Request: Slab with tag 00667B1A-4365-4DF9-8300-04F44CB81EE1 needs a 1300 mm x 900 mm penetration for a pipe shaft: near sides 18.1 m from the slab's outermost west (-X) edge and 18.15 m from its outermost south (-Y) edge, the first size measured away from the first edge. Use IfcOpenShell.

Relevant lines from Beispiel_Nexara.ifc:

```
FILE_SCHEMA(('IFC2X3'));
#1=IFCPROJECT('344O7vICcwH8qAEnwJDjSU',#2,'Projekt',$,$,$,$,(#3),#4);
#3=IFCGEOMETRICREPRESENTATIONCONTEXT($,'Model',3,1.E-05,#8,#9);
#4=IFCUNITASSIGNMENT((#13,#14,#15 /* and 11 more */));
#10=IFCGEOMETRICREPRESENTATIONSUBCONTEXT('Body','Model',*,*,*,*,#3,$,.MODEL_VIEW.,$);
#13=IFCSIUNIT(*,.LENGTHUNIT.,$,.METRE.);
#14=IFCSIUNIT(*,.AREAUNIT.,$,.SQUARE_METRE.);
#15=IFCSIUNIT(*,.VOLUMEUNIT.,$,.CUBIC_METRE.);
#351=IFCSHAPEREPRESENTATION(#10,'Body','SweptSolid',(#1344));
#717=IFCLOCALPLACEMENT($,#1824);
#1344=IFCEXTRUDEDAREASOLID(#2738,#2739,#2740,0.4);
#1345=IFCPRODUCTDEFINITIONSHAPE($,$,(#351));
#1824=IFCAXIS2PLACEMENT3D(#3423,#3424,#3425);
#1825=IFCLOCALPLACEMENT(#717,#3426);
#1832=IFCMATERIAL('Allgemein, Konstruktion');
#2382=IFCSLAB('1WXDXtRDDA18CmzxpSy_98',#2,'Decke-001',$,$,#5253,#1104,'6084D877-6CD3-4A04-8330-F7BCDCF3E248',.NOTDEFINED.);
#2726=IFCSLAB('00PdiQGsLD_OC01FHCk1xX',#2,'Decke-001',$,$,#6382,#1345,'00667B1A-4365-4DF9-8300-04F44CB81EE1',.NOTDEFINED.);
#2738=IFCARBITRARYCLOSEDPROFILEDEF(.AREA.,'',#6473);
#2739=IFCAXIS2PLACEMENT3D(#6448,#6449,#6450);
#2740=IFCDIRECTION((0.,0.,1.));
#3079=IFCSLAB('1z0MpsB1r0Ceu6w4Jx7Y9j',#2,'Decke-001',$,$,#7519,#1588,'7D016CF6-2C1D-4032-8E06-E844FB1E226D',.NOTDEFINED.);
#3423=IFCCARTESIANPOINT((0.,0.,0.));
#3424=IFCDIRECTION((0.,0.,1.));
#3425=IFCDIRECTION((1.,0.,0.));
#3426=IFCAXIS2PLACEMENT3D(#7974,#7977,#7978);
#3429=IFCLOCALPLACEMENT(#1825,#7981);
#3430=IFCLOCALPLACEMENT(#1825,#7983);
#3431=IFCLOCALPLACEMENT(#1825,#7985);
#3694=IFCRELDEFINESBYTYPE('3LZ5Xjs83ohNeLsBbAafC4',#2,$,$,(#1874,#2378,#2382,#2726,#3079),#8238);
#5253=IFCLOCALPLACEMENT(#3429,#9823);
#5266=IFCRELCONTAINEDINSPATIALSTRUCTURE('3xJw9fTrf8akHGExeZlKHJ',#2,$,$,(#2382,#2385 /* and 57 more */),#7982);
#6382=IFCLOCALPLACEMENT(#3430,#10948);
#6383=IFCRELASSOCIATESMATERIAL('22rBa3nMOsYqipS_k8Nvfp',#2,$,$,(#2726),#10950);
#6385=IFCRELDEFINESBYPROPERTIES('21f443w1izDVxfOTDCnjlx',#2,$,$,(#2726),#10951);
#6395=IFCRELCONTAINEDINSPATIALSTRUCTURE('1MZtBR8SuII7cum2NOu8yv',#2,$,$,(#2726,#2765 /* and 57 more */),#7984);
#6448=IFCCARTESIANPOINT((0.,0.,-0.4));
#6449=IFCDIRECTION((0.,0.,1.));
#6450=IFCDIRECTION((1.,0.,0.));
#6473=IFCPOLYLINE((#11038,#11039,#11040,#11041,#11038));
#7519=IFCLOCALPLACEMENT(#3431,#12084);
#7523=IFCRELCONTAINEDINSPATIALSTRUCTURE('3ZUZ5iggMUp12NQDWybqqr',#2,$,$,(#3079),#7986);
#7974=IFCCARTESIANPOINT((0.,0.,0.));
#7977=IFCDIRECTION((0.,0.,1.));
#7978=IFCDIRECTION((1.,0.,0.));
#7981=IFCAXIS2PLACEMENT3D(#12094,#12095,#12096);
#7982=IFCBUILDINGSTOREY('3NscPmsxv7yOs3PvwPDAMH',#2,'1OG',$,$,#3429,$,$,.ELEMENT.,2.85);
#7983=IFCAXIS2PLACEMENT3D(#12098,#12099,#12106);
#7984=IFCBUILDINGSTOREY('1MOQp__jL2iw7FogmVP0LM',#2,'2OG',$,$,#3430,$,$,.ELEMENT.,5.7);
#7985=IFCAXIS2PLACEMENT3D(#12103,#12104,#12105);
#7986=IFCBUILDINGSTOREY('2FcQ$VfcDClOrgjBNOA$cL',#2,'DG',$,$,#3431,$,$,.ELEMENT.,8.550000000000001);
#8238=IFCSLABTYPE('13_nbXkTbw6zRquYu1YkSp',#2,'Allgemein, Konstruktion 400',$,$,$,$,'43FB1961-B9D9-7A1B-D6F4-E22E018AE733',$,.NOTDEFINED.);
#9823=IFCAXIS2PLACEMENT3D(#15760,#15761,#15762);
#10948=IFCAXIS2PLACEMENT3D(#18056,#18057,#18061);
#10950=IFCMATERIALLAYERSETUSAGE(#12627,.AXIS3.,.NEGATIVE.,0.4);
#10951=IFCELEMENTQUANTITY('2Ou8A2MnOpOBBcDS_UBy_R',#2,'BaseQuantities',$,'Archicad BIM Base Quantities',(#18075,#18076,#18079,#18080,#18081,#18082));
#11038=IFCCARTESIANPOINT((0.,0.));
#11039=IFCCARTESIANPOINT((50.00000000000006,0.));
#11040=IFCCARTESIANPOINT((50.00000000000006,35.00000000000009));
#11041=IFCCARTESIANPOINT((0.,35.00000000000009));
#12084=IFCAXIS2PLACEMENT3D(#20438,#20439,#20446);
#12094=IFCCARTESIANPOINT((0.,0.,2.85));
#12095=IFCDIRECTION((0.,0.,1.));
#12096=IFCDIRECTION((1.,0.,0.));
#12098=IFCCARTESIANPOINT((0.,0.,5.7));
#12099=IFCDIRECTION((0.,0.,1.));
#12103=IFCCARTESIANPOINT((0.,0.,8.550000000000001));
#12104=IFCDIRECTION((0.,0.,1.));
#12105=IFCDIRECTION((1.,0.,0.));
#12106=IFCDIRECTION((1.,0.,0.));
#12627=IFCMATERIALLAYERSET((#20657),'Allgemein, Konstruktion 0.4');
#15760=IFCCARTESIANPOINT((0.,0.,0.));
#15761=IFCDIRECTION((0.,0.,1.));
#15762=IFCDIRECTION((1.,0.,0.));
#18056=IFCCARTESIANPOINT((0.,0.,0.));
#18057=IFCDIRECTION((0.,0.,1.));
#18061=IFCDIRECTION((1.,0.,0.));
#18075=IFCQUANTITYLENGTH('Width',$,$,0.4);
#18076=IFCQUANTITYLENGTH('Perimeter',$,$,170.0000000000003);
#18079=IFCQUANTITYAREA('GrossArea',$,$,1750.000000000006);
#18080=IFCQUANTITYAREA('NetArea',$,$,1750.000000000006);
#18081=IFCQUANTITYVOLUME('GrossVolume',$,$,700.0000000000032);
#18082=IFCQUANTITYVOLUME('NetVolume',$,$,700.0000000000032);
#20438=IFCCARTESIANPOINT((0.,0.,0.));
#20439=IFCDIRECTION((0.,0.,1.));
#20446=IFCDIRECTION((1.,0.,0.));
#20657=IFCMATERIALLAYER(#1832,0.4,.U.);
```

```python
import numpy as np
import ifcopenshell
import ifcopenshell.api.feature
import ifcopenshell.api.geometry
import ifcopenshell.api.pset
import ifcopenshell.api.root
import ifcopenshell.geom
import ifcopenshell.util.element
import ifcopenshell.util.placement
import ifcopenshell.util.representation
import ifcopenshell.util.shape
import ifcopenshell.util.unit

model = ifcopenshell.open("Beispiel_Nexara.ifc")
unit_scale = ifcopenshell.util.unit.calculate_unit_scale(model)
area_scale = ifcopenshell.util.unit.calculate_unit_scale(model, "AREAUNIT")
volume_scale = ifcopenshell.util.unit.calculate_unit_scale(model, "VOLUMEUNIT")
settings = ifcopenshell.geom.settings()


def volume(element):
    """Net volume in cubic metres, openings subtracted."""
    shape = ifcopenshell.geom.create_shape(settings, element)
    return ifcopenshell.util.shape.get_volume(shape.geometry)


slab = model.by_guid("00PdiQGsLD_OC01FHCk1xX")
before = volume(slab)

# Extent in the slab's own axes, in metres. The edges named are its -X and -Y sides.
slab_shape = ifcopenshell.geom.create_shape(settings, slab)
vertices = ifcopenshell.util.shape.get_vertices(slab_shape.geometry)
x_min, y_min, bottom = vertices.min(axis=0)
top = vertices[:, 2].max()

opening = ifcopenshell.api.root.create_entity(model, ifc_class="IfcOpeningElement", name="Pipe shaft opening")
context = ifcopenshell.util.representation.get_context(model, "Model", "Body", "MODEL_VIEW")
width, depth = 1.3, 0.9
outline = [(0.0, 0.0), (width, 0.0), (width, depth), (0.0, depth), (0.0, 0.0)]
# Overshoot both faces by 50 mm so the cut is clean.
shape = ifcopenshell.api.geometry.add_slab_representation(
    model, context=context, depth=top - bottom + 0.1, polyline=outline
)
ifcopenshell.api.geometry.assign_representation(model, product=opening, representation=shape)

matrix = ifcopenshell.util.placement.get_local_placement(slab.ObjectPlacement)
matrix[:, 3] = matrix @ np.append(np.array([x_min + 18.1, y_min + 18.15, bottom - 0.05]) / unit_scale, 1.0)
ifcopenshell.api.geometry.edit_object_placement(model, product=opening, matrix=matrix, is_si=False)
ifcopenshell.api.feature.add_feature(model, feature=opening, element=slab)

after = volume(slab)

# Update the slab's stored quantities.
qto = model.by_id(ifcopenshell.util.element.get_pset(slab, "BaseQuantities", should_inherit=False)["id"])
ifcopenshell.api.pset.edit_qto(model, qto=qto, properties={
    "NetArea": after / (top - bottom) / area_scale,
    "NetVolume": after / volume_scale,
})

print(f"slab volume {before:.3f} -> {after:.3f} m3")

model.write("Beispiel_Nexara_v2.ifc")
```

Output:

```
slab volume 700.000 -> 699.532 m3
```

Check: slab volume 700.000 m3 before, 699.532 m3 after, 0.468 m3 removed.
